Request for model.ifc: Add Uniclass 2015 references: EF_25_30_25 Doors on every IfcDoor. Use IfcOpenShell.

First a look at what the model holds.

```python
import ifcopenshell

model = ifcopenshell.open("model.ifc")
print(model.schema)
print("classifications:", [c.Name for c in model.by_type("IfcClassification")])
for ifc_class in ("IfcDoor", "IfcRoof", "IfcStair", "IfcWall", "IfcWindow"):
    print(ifc_class, len(model.by_type(ifc_class)))
```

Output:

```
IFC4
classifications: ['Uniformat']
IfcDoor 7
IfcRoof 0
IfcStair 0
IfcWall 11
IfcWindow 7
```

```python
import ifcopenshell
import ifcopenshell.api.classification

model = ifcopenshell.open("model.ifc")

system = ifcopenshell.api.classification.add_classification(model, classification="Uniclass 2015")

codes = {
    "IfcDoor": ("EF_25_30_25", "Doors"),
}
for ifc_class, (code, name) in codes.items():
    products = model.by_type(ifc_class)
    ifcopenshell.api.classification.add_reference(
        model, products=products, classification=system, identification=code, name=name
    )
    print(code, len(products))

model.write("model-out.ifc")
```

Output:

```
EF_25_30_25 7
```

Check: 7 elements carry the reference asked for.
